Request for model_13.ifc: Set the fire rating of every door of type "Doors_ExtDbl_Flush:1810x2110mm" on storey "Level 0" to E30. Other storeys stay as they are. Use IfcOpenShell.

First a look at what the model holds.

```python
import ifcopenshell
import ifcopenshell.util.element

model = ifcopenshell.open("model_13.ifc")
print(model.schema)
storey = next(s for s in model.by_type("IfcBuildingStorey") if s.Name == "Level 0")
doors = [e for e in ifcopenshell.util.element.get_decomposition(storey) if e.is_a("IfcDoor")]
seen = {}
for e in doors:
    element_type = ifcopenshell.util.element.get_type(e)
    key = (element_type.Name if element_type != e and element_type else None, ifcopenshell.util.element.get_pset(e, "Pset_DoorCommon", "FireRating"))
    seen[key] = seen.get(key, 0) + 1
for (name, value), count in sorted(seen.items(), key=str):
    print(count, "x", name, "|", value)
```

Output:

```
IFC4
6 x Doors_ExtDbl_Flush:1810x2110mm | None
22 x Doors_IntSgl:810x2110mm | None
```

```python
import ifcopenshell
import ifcopenshell.api.pset
import ifcopenshell.util.element

model = ifcopenshell.open("model_13.ifc")

storey = next(s for s in model.by_type("IfcBuildingStorey") if s.Name == "Level 0")
doors = [e for e in ifcopenshell.util.element.get_decomposition(storey) if e.is_a("IfcDoor")]

count = 0
for e in doors:
    element_type = ifcopenshell.util.element.get_type(e)
    if element_type in (None, e) or element_type.Name != "Doors_ExtDbl_Flush:1810x2110mm":
        continue
    # add_pset returns the element's existing set when there is one.
    pset = ifcopenshell.api.pset.add_pset(model, product=e, name="Pset_DoorCommon")
    ifcopenshell.api.pset.edit_pset(model, pset=pset, properties={"FireRating": "E30"})
    count += 1

print(count, "doors updated")

model.write("model_13_rev.ifc")
```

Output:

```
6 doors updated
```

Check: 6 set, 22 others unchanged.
